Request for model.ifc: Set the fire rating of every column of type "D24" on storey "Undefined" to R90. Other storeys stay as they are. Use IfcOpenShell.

First a look at what the model holds.

```python
import ifcopenshell
import ifcopenshell.util.element

model = ifcopenshell.open("model.ifc")
print(model.schema)
storey = next(s for s in model.by_type("IfcBuildingStorey") if s.Name == "Undefined")
columns = [e for e in ifcopenshell.util.element.get_decomposition(storey) if e.is_a("IfcColumn")]
seen = {}
for e in columns:
    element_type = ifcopenshell.util.element.get_type(e)
    key = (element_type.Name if element_type != e and element_type else None, ifcopenshell.util.element.get_pset(e, "Pset_ColumnCommon", "FireRating"))
    seen[key] = seen.get(key, 0) + 1
for (name, value), count in sorted(seen.items(), key=str):
    print(count, "x", name, "|", value)
```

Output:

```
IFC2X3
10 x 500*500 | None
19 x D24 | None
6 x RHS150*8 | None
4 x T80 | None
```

```python
import ifcopenshell
import ifcopenshell.api.pset
import ifcopenshell.util.element

model = ifcopenshell.open("model.ifc")

storey = next(s for s in model.by_type("IfcBuildingStorey") if s.Name == "Undefined")
columns = [e for e in ifcopenshell.util.element.get_decomposition(storey) if e.is_a("IfcColumn")]

count = 0
for e in columns:
    element_type = ifcopenshell.util.element.get_type(e)
    if element_type in (None, e) or element_type.Name != "D24":
        continue
    # add_pset returns the element's existing set when there is one.
    pset = ifcopenshell.api.pset.add_pset(model, product=e, name="Pset_ColumnCommon")
    ifcopenshell.api.pset.edit_pset(model, pset=pset, properties={"FireRating": "R90"})
    count += 1

print(count, "columns updated")

model.write("model_updated.ifc")
```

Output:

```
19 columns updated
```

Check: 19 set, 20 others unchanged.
